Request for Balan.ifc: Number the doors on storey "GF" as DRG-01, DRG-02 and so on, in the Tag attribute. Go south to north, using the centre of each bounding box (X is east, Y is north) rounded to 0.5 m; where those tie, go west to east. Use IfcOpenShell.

First a look at what the model holds.

```python
import ifcopenshell
import ifcopenshell.util.element
import ifcopenshell.util.placement

model = ifcopenshell.open("Balan.ifc")
print(model.schema)
storey = next(s for s in model.by_type("IfcBuildingStorey") if s.Name == "GF")
doors = [e for e in ifcopenshell.util.element.get_decomposition(storey) if e.is_a("IfcDoor")]
for e in sorted(doors, key=lambda e: e.id()):
    origin = ifcopenshell.util.placement.get_local_placement(e.ObjectPlacement)[:3, 3]
    print(e.id(), e.Tag, e.Name, origin.round(2) + 0.0, sep=" | ")
```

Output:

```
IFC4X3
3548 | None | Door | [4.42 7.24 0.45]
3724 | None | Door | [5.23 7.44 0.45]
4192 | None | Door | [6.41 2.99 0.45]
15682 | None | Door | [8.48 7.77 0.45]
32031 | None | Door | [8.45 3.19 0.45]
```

```python
import ifcopenshell
import ifcopenshell.geom
import ifcopenshell.util.element
import ifcopenshell.util.shape

model = ifcopenshell.open("Balan.ifc")
settings = ifcopenshell.geom.settings()
settings.set("use-world-coords", True)


def centre(element):
    shape = ifcopenshell.geom.create_shape(settings, element)
    return ifcopenshell.util.shape.get_bbox_centroid(shape.geometry)


storey = next(s for s in model.by_type("IfcBuildingStorey") if s.Name == "GF")
doors = [e for e in ifcopenshell.util.element.get_decomposition(storey) if e.is_a("IfcDoor")]

# Insertion points can sit at a corner or the storey origin, so sort by the geometry (in metres).
centres = {e: centre(e) for e in doors}
doors.sort(key=lambda e: (round(centres[e][1] / 0.5), centres[e][0]))

for i, e in enumerate(doors, start=1):
    number = f"DRG-{i:02d}"
    e.Tag = number
    print(e.id(), number)

model.write("Balan-out.ifc")
```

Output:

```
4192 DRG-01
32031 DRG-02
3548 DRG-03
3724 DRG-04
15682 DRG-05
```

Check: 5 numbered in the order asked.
